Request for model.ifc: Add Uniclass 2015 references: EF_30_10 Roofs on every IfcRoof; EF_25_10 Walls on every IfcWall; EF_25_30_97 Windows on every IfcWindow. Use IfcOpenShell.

First a look at what the model holds.

```python
import ifcopenshell

model = ifcopenshell.open("model.ifc")
print(model.schema)
print("classifications:", [c.Name for c in model.by_type("IfcClassification")])
for ifc_class in ("IfcDoor", "IfcRoof", "IfcStair", "IfcWall", "IfcWindow"):
    print(ifc_class, len(model.by_type(ifc_class)))
```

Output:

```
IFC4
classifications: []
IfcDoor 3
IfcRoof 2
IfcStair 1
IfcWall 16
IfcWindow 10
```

```python
import ifcopenshell
import ifcopenshell.api.classification

model = ifcopenshell.open("model.ifc")

system = ifcopenshell.api.classification.add_classification(model, classification="Uniclass 2015")

codes = {
    "IfcRoof": ("EF_30_10", "Roofs"),
    "IfcWall": ("EF_25_10", "Walls"),
    "IfcWindow": ("EF_25_30_97", "Windows"),
}
for ifc_class, (code, name) in codes.items():
    products = model.by_type(ifc_class)
    ifcopenshell.api.classification.add_reference(
        model, products=products, classification=system, identification=code, name=name
    )
    print(code, len(products))

model.write("model_rev.ifc")
```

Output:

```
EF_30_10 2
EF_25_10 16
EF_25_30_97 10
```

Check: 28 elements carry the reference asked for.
